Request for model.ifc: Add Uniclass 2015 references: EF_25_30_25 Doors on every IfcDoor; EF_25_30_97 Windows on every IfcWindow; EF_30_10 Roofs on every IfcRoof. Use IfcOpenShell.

First a look at what the model holds.

```python
import ifcopenshell

model = ifcopenshell.open("model.ifc")
print(model.schema)
print("classifications:", [c.Name for c in model.by_type("IfcClassification")])
for ifc_class in ("IfcDoor", "IfcRoof", "IfcStair", "IfcWall", "IfcWindow"):
    print(ifc_class, len(model.by_type(ifc_class)))
```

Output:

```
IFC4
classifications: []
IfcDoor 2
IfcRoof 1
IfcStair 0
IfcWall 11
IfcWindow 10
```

```python
import ifcopenshell
import ifcopenshell.api.classification

model = ifcopenshell.open("model.ifc")

system = ifcopenshell.api.classification.add_classification(model, classification="Uniclass 2015")

codes = {
    "IfcDoor": ("EF_25_30_25", "Doors"),
    "IfcWindow": ("EF_25_30_97", "Windows"),
    "IfcRoof": ("EF_30_10", "Roofs"),
}
for ifc_class, (code, name) in codes.items():
    products = model.by_type(ifc_class)
    ifcopenshell.api.classification.add_reference(
        model, products=products, classification=system, identification=code, name=name
    )
    print(code, len(products))

model.write("model_updated.ifc")
```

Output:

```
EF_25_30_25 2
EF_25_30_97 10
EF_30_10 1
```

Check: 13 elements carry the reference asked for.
